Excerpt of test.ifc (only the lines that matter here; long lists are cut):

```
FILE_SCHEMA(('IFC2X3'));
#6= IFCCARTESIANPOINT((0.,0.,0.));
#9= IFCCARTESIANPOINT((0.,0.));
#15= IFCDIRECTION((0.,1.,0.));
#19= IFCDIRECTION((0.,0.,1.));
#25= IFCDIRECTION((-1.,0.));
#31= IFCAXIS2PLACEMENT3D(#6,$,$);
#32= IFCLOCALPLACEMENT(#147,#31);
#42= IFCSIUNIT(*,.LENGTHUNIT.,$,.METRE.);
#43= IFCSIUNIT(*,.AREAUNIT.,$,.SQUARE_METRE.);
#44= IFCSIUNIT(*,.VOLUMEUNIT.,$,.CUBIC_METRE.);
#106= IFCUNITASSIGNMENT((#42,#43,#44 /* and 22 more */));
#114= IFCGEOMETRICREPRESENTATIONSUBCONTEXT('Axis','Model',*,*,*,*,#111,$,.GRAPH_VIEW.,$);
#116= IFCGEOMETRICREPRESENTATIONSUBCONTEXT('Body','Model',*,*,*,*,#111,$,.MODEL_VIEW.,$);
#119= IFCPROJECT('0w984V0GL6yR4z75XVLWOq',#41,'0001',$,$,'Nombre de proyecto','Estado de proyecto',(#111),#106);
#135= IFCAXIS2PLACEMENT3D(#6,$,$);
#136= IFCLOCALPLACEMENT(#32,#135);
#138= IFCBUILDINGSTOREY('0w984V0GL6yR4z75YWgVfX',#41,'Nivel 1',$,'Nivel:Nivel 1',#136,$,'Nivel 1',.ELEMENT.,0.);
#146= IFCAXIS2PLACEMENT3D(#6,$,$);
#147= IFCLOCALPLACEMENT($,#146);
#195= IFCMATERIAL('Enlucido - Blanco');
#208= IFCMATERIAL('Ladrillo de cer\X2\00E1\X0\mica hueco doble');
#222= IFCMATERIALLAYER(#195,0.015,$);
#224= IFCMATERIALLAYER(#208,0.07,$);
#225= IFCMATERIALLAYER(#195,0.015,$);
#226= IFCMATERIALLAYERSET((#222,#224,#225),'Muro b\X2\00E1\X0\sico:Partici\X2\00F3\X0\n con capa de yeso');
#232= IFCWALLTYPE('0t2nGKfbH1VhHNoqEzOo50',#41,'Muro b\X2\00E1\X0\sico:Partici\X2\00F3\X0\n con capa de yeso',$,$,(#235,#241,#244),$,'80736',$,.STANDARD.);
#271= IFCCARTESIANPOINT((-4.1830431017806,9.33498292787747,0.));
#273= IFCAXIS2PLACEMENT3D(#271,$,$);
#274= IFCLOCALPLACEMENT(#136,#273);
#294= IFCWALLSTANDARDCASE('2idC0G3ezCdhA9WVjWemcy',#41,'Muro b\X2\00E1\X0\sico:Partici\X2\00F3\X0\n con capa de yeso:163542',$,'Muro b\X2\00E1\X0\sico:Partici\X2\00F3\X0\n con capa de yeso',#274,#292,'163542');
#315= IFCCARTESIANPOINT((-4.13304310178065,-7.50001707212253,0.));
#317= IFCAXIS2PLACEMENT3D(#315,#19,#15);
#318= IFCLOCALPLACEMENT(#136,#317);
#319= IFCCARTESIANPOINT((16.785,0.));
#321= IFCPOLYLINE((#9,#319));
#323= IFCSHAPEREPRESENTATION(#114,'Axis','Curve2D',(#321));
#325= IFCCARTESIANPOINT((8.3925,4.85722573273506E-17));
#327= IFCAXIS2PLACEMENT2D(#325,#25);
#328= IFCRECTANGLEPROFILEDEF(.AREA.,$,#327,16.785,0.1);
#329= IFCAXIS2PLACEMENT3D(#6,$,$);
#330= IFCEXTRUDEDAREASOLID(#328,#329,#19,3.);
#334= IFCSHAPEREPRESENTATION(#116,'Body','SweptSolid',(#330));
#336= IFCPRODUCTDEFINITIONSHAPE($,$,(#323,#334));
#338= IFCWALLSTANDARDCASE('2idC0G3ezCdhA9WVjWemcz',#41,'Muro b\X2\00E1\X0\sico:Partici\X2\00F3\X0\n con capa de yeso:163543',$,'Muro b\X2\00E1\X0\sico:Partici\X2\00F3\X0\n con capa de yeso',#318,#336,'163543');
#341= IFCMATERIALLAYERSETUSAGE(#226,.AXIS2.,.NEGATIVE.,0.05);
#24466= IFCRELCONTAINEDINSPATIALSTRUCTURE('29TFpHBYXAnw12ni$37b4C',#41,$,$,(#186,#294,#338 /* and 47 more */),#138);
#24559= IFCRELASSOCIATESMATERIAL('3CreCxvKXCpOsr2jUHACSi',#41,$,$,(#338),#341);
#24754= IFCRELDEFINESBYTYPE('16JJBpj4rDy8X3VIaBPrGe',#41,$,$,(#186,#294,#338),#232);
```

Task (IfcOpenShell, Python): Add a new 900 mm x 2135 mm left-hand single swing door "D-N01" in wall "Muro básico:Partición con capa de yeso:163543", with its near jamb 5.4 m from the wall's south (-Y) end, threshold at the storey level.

```python
import numpy as np
import ifcopenshell
import ifcopenshell.api.feature
import ifcopenshell.api.geometry
import ifcopenshell.api.root
import ifcopenshell.api.spatial
import ifcopenshell.api.type
import ifcopenshell.geom
import ifcopenshell.util.element
import ifcopenshell.util.placement
import ifcopenshell.util.representation
import ifcopenshell.util.shape
import ifcopenshell.util.unit

model = ifcopenshell.open("test.ifc")
unit_scale = ifcopenshell.util.unit.calculate_unit_scale(model)
settings = ifcopenshell.geom.settings()


def volume(element):
    """Net volume in cubic metres, openings subtracted."""
    shape = ifcopenshell.geom.create_shape(settings, element)
    return ifcopenshell.util.shape.get_volume(shape.geometry)


wall = model.by_id(338)
storey = ifcopenshell.util.element.get_container(wall, ifc_class="IfcBuildingStorey")
context = ifcopenshell.util.representation.get_context(model, "Model", "Body", "MODEL_VIEW")
before = volume(wall)

width, height, from_end, sill = 0.9, 2.135, 5.4, 0.0  # metres

# The wall runs along its own X axis, and the end named is its -X end.
wall_shape = ifcopenshell.geom.create_shape(settings, wall)
x, y, z = ifcopenshell.util.shape.get_vertices(wall_shape.geometry).T
start = x.min() + from_end
face, thickness = float(y.min()), float(y.max() - y.min())
wall_matrix = ifcopenshell.util.placement.get_local_placement(wall.ObjectPlacement)
level = ifcopenshell.util.placement.get_local_placement(storey.ObjectPlacement)[2, 3]


def in_wall(x, y):
    """Placement at x, y metres in the wall's axes, at sill height."""
    matrix = wall_matrix.copy()
    matrix[:, 3] = wall_matrix @ np.array([x / unit_scale, y / unit_scale, 0.0, 1.0])
    matrix[2, 3] = level + sill / unit_scale
    return matrix


# Opening: a box that overshoots both wall faces by 50 mm.
opening = ifcopenshell.api.root.create_entity(model, ifc_class="IfcOpeningElement")
box = ifcopenshell.api.geometry.add_wall_representation(
    model, context=context, length=width, height=height, thickness=thickness + 0.1
)
ifcopenshell.api.geometry.assign_representation(model, product=opening, representation=box)
ifcopenshell.api.geometry.edit_object_placement(model, product=opening, matrix=in_wall(start, face - 0.05), is_si=False)
ifcopenshell.api.feature.add_feature(model, feature=opening, element=wall)

door = ifcopenshell.api.root.create_entity(model, ifc_class="IfcDoor", name="D-N01")
door.OverallWidth, door.OverallHeight = width / unit_scale, height / unit_scale
body = ifcopenshell.api.geometry.add_door_representation(
    model,
    context=context,
    overall_width=door.OverallWidth,
    overall_height=door.OverallHeight,
    operation_type="SINGLE_SWING_LEFT",
    lining_properties={"LiningDepth": thickness / unit_scale, "ThresholdDepth": thickness / unit_scale},
)
ifcopenshell.api.geometry.assign_representation(model, product=door, representation=body)
ifcopenshell.api.spatial.assign_container(model, products=[door], relating_structure=storey)
fills = ifcopenshell.api.feature.add_filling(model, opening=opening, element=door)
fills.OwnerHistory = door.OwnerHistory  # required in IFC2X3

# IFC2X3 keeps the operation on the door style.
style = ifcopenshell.api.root.create_entity(model, ifc_class="IfcDoorStyle", name="D-N01")
style.OperationType, style.ConstructionType = "SINGLE_SWING_LEFT", "NOTDEFINED"
style.ParameterTakesPrecedence = style.Sizeable = False
ifcopenshell.api.type.assign_type(model, related_objects=[door], relating_type=style)

# The lining spans the wall, so the door starts at the wall face.
ifcopenshell.api.geometry.edit_object_placement(model, product=door, matrix=in_wall(start, face), is_si=False)

after = volume(wall)

print(f"wall volume {before:.3f} -> {after:.3f} m3")

model.write("test_rev.ifc")
```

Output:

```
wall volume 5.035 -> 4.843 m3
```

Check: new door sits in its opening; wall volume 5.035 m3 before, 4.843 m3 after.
